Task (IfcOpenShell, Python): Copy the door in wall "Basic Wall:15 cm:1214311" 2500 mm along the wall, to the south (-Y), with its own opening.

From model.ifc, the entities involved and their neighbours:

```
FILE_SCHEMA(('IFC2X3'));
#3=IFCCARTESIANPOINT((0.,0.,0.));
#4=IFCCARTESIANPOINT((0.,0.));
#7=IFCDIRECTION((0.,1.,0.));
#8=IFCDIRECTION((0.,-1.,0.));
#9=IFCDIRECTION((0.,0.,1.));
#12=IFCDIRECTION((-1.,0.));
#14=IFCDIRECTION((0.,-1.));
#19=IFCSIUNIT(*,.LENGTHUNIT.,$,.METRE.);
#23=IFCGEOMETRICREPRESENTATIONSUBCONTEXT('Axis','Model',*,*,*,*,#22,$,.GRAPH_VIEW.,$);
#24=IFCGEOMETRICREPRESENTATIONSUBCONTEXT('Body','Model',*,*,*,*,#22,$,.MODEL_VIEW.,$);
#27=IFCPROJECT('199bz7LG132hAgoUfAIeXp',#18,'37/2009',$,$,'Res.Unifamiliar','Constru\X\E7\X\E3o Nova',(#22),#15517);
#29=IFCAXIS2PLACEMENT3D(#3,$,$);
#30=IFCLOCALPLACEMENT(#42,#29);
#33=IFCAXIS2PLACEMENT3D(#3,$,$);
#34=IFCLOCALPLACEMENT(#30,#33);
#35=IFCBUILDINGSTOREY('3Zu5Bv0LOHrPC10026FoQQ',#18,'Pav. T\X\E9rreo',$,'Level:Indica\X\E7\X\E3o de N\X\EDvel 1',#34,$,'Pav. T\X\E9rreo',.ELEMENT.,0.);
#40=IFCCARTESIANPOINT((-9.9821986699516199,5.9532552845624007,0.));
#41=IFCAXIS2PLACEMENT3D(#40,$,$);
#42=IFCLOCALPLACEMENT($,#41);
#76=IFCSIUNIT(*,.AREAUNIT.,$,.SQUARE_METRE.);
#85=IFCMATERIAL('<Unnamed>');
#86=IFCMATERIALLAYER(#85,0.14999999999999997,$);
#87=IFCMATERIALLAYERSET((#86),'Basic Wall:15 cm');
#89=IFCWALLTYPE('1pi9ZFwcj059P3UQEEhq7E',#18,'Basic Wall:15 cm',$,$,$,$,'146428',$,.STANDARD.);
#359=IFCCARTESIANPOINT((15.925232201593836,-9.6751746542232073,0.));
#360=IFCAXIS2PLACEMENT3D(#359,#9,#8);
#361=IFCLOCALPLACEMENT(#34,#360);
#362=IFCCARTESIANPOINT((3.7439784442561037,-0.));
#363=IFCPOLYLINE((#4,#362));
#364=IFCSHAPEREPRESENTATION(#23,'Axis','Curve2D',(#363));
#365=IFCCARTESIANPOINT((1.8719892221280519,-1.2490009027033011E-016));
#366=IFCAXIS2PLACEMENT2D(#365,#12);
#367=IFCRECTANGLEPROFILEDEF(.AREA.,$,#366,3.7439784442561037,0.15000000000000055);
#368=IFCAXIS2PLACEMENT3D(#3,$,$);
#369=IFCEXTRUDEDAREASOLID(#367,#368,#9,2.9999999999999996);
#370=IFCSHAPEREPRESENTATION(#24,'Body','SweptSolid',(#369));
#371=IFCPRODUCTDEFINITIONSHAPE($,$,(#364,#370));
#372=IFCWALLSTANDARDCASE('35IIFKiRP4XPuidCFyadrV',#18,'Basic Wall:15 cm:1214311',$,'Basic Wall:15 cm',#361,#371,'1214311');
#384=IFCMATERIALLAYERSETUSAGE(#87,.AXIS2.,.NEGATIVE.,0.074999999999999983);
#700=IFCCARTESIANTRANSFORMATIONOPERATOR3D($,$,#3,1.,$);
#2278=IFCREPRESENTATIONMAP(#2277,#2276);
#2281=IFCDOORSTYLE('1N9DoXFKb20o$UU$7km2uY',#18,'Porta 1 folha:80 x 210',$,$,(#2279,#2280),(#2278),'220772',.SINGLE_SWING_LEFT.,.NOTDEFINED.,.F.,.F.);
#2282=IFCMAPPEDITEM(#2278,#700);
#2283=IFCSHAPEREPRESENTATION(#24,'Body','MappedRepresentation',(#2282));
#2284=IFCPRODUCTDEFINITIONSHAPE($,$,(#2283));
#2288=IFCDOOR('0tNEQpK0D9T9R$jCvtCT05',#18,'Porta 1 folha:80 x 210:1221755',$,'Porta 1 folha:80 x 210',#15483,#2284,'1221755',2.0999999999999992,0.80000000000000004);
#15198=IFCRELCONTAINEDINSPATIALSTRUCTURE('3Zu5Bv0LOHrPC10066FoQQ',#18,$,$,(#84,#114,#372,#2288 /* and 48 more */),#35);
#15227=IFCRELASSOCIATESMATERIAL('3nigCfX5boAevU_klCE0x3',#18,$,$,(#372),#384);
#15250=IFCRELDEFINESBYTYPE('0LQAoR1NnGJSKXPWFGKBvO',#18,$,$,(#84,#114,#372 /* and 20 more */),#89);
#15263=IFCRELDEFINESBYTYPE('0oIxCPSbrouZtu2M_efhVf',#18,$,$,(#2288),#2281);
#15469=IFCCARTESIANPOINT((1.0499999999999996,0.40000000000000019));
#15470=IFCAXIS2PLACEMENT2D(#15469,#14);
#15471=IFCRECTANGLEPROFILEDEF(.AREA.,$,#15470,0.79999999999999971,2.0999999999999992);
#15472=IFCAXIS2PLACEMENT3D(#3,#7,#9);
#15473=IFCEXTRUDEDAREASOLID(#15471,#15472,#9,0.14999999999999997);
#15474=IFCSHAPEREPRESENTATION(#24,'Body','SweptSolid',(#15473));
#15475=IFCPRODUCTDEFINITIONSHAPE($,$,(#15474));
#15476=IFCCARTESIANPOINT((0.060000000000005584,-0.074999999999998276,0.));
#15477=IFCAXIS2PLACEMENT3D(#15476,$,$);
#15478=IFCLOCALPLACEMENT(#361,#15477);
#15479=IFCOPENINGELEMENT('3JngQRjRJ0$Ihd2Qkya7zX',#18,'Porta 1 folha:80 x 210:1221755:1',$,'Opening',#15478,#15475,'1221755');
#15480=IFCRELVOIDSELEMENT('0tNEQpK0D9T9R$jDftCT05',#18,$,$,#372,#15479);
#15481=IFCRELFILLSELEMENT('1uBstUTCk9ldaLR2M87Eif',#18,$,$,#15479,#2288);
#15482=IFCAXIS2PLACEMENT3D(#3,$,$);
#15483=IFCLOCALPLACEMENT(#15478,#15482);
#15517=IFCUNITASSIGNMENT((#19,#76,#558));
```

```python
import ifcopenshell
import ifcopenshell.api.feature
import ifcopenshell.api.geometry
import ifcopenshell.api.root
import ifcopenshell.geom
import ifcopenshell.util.element
import ifcopenshell.util.placement
import ifcopenshell.util.shape

model = ifcopenshell.open("model.ifc")
settings = ifcopenshell.geom.settings()


def volume(element):
    """Net volume in cubic metres, openings subtracted."""
    shape = ifcopenshell.geom.create_shape(settings, element)
    return ifcopenshell.util.shape.get_volume(shape.geometry)


def reuse_history(source, copy):
    """copy_class also copies each property set's owner history, people and application; keep the originals."""
    for rel in copy.IsDefinedBy:
        if rel.is_a("IfcRelDefinesByProperties") and (history := rel.RelatingPropertyDefinition.OwnerHistory):
            rel.RelatingPropertyDefinition.OwnerHistory = source.OwnerHistory
            ifcopenshell.util.element.remove_deep2(model, history)


door = model.by_id(2288)
opening = door.FillsVoids[0].RelatingOpeningElement
wall = opening.VoidsElements[0].RelatingBuildingElement
before = volume(wall)
shift = ifcopenshell.util.placement.get_local_placement(wall.ObjectPlacement)[:3, 0] * 2.5

# copy_class copies the void relationship, type, container and properties, but no geometry.
new_opening = ifcopenshell.api.root.copy_class(model, product=opening)
new_opening.Representation = ifcopenshell.util.element.copy_deep(
    model, opening.Representation, exclude=["IfcGeometricRepresentationContext", "IfcRepresentationMap"]
)
new_opening.Name = "Porta 1 folha:80 x 210"
new_opening.Tag = None
new_door = ifcopenshell.api.root.copy_class(model, product=door)
new_door.Representation = ifcopenshell.util.element.copy_deep(
    model, door.Representation, exclude=["IfcGeometricRepresentationContext", "IfcRepresentationMap"]
)
new_door.Name = "Porta 1 folha:80 x 210"
new_door.Tag = None
reuse_history(door, new_door)
fills = ifcopenshell.api.feature.add_filling(model, opening=new_opening, element=new_door)
fills.OwnerHistory = new_door.OwnerHistory  # required in IFC2X3

for old, new in ((opening, new_opening), (door, new_door)):
    matrix = ifcopenshell.util.placement.get_local_placement(old.ObjectPlacement)
    matrix[:3, 3] += shift
    ifcopenshell.api.geometry.edit_object_placement(model, product=new, matrix=matrix, is_si=False)

after = volume(wall)

print(f"wall volume {before:.3f} -> {after:.3f} m3")

model.write("model_rev.ifc")
```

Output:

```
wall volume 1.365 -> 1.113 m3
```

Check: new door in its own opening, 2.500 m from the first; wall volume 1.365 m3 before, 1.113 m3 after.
